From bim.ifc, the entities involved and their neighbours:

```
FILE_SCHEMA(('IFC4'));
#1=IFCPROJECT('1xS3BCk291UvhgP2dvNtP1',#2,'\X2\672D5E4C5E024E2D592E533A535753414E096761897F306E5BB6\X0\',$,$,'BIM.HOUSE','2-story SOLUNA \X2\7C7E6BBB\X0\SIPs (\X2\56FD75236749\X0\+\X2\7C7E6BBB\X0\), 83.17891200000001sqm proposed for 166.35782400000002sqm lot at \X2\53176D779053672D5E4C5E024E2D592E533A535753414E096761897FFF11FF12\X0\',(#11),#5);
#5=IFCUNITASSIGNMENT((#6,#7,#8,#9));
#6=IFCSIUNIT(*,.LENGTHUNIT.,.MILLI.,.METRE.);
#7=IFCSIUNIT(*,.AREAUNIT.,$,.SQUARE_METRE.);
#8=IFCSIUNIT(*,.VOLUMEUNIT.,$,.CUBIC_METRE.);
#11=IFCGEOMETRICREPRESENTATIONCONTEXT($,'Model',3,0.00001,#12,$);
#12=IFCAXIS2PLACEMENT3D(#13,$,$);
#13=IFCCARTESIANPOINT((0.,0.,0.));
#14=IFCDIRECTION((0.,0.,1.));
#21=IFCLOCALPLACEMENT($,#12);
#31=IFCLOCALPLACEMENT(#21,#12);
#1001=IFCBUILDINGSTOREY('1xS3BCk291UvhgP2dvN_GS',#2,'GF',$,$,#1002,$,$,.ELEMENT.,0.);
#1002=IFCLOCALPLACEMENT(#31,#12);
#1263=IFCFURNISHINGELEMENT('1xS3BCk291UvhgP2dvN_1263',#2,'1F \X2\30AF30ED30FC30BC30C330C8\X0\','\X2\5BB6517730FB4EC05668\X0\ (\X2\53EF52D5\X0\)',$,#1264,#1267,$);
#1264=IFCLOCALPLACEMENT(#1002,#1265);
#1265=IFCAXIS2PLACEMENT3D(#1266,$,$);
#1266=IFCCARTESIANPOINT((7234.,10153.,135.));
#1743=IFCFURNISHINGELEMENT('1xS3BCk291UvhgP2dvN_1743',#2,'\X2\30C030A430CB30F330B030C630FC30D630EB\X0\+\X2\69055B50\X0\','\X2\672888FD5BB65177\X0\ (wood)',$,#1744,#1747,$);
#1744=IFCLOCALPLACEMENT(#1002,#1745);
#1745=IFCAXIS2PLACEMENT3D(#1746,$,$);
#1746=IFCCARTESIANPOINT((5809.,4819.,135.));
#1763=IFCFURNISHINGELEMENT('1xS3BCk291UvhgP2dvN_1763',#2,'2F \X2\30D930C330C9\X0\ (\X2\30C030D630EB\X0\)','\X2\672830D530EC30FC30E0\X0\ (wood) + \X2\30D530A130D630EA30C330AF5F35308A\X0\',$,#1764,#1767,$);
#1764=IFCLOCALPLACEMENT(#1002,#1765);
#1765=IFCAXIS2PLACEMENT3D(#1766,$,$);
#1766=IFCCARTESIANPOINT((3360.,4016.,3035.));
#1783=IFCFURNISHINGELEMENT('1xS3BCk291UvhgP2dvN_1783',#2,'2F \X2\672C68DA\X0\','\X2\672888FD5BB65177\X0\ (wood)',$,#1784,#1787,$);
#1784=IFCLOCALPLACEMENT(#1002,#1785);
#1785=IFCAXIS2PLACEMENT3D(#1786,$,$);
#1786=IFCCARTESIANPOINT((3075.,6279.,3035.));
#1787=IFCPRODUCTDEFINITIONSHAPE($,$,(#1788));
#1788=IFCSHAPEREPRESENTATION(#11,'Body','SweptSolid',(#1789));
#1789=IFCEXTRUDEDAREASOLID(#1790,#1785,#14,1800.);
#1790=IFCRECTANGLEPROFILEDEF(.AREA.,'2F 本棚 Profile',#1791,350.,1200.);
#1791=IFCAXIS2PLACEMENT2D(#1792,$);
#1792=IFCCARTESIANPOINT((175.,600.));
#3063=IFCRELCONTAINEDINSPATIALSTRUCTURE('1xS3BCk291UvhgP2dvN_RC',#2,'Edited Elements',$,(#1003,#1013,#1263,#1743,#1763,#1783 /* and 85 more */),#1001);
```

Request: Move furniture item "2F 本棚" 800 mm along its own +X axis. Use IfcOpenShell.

```python
import ifcopenshell
import ifcopenshell.api.geometry
import ifcopenshell.util.placement

model = ifcopenshell.open("bim.ifc")

item = model.by_id(1783)
matrix = ifcopenshell.util.placement.get_local_placement(item.ObjectPlacement)
matrix[:3, 3] += matrix[:3, 0] * 800.0
ifcopenshell.api.geometry.edit_object_placement(model, product=item, matrix=matrix, is_si=False)

print(ifcopenshell.util.placement.get_local_placement(item.ObjectPlacement).round(3) + 0.0)

model.write("bim-out.ifc")
```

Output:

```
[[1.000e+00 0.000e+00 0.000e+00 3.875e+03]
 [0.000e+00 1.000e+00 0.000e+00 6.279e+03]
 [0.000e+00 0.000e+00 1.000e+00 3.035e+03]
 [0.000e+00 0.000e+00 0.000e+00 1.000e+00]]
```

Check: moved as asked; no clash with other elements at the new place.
